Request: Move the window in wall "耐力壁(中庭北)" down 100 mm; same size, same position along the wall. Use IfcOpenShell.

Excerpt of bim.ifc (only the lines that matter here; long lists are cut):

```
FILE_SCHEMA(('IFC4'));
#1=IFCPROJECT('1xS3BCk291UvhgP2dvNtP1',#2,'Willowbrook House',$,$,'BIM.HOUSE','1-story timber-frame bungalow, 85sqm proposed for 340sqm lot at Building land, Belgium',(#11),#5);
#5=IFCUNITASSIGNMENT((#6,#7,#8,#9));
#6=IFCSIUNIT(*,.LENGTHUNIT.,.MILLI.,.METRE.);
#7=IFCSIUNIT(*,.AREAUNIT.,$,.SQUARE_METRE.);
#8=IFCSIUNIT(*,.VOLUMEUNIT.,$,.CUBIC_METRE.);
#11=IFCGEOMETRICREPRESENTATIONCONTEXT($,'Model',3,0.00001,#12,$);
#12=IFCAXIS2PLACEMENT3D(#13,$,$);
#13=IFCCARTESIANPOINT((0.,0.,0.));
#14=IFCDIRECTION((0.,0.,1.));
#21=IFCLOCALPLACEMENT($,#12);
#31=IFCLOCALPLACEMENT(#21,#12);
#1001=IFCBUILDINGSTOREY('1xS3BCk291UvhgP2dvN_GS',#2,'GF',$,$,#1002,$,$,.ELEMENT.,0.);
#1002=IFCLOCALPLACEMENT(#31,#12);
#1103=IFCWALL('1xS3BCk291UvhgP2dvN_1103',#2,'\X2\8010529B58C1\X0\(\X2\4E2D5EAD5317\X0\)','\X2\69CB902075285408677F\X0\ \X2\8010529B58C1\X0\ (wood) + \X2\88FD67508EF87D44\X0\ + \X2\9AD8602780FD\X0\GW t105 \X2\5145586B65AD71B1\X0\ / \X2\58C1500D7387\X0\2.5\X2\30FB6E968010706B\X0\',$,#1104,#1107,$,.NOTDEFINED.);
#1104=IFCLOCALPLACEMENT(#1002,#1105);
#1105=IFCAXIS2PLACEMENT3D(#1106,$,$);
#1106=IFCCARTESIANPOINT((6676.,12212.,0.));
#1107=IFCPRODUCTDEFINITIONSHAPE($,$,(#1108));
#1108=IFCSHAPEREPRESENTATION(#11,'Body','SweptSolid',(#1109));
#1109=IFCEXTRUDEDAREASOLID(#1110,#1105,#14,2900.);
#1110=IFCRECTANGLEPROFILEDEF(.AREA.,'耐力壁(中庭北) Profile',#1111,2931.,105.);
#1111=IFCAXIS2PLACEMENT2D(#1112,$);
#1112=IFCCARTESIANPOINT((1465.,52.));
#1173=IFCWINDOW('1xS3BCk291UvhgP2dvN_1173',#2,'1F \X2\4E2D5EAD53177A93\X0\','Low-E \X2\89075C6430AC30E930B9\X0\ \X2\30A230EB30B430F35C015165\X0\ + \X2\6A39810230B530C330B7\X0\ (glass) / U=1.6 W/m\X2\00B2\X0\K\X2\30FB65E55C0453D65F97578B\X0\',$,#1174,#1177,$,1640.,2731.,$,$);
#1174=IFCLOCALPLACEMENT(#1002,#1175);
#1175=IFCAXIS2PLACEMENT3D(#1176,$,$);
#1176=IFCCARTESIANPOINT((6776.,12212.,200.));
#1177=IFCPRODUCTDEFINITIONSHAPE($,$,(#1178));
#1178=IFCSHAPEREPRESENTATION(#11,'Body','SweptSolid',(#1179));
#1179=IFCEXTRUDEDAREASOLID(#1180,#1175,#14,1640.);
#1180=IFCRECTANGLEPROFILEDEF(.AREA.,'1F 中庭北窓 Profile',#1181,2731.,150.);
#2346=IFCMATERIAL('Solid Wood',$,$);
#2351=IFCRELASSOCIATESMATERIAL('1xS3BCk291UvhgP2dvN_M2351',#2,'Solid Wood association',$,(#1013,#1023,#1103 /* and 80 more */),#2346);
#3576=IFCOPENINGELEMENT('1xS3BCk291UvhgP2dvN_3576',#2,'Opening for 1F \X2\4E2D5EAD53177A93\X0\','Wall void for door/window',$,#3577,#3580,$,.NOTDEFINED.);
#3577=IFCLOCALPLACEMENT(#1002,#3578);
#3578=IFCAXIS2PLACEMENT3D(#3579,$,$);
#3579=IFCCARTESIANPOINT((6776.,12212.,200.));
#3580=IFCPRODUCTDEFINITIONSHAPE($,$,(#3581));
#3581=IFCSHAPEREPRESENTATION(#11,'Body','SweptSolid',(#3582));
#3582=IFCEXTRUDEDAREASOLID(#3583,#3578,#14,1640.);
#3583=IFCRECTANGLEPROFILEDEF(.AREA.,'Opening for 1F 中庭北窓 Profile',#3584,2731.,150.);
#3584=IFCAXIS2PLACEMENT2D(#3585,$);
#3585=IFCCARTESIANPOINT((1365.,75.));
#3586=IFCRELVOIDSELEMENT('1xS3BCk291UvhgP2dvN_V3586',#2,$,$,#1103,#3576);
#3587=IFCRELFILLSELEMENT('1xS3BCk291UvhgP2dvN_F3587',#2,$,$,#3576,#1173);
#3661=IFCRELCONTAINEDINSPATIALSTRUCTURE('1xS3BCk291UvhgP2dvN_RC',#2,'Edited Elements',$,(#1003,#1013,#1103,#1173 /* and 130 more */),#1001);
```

```python
import numpy as np
import ifcopenshell
import ifcopenshell.api.geometry
import ifcopenshell.util.placement
import ifcopenshell.util.unit

model = ifcopenshell.open("bim.ifc")
unit_scale = ifcopenshell.util.unit.calculate_unit_scale(model)

window = model.by_guid("1xS3BCk291UvhgP2dvN_1173")
opening = window.FillsVoids[0].RelatingOpeningElement
dz = -0.1 / unit_scale

shift = np.array([0.0, 0.0, dz])
# The window is not placed relative to its opening, so move both.
for product in (opening, window):
    matrix = ifcopenshell.util.placement.get_local_placement(product.ObjectPlacement)
    matrix[:3, 3] += shift
    ifcopenshell.api.geometry.edit_object_placement(model, product=product, matrix=matrix, is_si=False)

print(f"moved by {dz * unit_scale:+.3f} m")

model.write("bim_updated.ifc")
```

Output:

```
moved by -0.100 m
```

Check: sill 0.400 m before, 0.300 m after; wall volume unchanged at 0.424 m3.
